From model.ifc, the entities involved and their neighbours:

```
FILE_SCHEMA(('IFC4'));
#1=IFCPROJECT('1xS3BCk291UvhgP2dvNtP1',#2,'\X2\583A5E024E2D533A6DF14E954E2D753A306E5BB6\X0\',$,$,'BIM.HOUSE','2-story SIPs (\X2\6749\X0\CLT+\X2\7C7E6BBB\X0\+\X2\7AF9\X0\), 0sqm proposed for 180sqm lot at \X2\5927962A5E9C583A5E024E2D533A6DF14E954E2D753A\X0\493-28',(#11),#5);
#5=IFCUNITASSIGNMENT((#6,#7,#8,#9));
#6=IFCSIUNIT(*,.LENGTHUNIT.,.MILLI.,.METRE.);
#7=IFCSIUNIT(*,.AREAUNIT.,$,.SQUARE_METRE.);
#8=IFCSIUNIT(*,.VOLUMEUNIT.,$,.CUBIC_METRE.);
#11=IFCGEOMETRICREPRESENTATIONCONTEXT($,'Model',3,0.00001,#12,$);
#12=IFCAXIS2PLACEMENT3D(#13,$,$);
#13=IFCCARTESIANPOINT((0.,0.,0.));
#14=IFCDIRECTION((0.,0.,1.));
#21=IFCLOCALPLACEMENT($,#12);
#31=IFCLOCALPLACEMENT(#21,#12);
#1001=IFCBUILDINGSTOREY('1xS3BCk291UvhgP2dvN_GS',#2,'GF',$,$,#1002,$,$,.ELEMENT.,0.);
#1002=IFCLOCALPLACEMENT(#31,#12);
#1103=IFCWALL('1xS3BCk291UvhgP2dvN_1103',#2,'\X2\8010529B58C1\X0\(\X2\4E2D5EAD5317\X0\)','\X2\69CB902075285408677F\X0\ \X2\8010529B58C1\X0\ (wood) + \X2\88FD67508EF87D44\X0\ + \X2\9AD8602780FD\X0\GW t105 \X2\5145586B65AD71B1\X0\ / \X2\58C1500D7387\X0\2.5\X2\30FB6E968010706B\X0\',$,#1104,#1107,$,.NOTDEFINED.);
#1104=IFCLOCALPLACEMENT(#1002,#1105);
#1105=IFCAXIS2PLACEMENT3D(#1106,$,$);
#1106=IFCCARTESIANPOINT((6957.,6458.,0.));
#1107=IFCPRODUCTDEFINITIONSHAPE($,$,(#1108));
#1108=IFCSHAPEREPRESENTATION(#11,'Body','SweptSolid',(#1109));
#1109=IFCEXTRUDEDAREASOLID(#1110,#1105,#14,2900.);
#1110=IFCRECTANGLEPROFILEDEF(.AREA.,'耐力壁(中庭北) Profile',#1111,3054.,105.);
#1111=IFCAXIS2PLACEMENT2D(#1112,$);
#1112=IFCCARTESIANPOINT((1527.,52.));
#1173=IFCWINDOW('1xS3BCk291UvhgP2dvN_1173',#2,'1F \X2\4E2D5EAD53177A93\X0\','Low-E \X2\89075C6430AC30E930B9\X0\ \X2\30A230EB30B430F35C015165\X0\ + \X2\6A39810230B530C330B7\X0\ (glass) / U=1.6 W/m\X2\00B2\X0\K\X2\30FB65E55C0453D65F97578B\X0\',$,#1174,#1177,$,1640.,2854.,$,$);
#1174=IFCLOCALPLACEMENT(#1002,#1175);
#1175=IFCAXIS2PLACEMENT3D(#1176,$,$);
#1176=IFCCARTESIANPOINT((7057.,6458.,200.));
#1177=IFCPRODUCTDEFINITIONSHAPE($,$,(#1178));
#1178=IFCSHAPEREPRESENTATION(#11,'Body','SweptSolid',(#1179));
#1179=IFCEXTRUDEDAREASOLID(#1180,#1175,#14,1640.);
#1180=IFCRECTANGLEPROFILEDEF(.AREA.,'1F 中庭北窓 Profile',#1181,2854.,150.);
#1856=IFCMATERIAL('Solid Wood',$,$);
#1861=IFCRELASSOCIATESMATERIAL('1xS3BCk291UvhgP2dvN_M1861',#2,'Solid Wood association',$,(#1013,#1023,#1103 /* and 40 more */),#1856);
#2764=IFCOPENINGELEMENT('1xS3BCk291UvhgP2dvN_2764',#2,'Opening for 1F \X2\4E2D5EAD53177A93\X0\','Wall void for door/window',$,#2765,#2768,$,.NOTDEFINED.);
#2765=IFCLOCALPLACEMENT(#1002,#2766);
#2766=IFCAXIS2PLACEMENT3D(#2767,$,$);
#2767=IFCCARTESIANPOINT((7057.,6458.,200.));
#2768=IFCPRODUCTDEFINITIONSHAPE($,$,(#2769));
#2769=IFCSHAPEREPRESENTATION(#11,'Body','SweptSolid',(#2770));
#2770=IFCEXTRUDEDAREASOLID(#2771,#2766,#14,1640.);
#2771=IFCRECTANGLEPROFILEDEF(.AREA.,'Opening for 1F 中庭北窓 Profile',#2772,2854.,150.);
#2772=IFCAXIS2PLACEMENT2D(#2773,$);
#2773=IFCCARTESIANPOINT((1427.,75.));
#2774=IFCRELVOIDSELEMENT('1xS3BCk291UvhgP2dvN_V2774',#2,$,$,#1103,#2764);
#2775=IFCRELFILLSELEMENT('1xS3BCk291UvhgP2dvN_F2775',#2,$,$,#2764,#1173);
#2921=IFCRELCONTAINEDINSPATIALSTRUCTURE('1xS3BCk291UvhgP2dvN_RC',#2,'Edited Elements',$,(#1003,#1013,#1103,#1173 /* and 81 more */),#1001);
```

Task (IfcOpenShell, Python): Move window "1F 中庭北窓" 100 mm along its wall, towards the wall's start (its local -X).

```python
import ifcopenshell
import ifcopenshell.api.geometry
import ifcopenshell.util.placement
import ifcopenshell.util.unit

model = ifcopenshell.open("model.ifc")
unit_scale = ifcopenshell.util.unit.calculate_unit_scale(model)

window = model.by_id(1173)
opening = window.FillsVoids[0].RelatingOpeningElement
wall = opening.VoidsElements[0].RelatingBuildingElement

wall_matrix = ifcopenshell.util.placement.get_local_placement(wall.ObjectPlacement)
shift = wall_matrix[:3, 0] * -0.1 / unit_scale
before = ifcopenshell.util.placement.get_local_placement(window.ObjectPlacement)[:3, 3].copy()

# The window is not placed relative to its opening, so move both.
for product in (opening, window):
    matrix = ifcopenshell.util.placement.get_local_placement(product.ObjectPlacement)
    matrix[:3, 3] += shift
    ifcopenshell.api.geometry.edit_object_placement(model, product=product, matrix=matrix, is_si=False)

after = ifcopenshell.util.placement.get_local_placement(window.ObjectPlacement)[:3, 3]
print("window moved by", (after - before).round(3) + 0.0)

model.write("model_v2.ifc")
```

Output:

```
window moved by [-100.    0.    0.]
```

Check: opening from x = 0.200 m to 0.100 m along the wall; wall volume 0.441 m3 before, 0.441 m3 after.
